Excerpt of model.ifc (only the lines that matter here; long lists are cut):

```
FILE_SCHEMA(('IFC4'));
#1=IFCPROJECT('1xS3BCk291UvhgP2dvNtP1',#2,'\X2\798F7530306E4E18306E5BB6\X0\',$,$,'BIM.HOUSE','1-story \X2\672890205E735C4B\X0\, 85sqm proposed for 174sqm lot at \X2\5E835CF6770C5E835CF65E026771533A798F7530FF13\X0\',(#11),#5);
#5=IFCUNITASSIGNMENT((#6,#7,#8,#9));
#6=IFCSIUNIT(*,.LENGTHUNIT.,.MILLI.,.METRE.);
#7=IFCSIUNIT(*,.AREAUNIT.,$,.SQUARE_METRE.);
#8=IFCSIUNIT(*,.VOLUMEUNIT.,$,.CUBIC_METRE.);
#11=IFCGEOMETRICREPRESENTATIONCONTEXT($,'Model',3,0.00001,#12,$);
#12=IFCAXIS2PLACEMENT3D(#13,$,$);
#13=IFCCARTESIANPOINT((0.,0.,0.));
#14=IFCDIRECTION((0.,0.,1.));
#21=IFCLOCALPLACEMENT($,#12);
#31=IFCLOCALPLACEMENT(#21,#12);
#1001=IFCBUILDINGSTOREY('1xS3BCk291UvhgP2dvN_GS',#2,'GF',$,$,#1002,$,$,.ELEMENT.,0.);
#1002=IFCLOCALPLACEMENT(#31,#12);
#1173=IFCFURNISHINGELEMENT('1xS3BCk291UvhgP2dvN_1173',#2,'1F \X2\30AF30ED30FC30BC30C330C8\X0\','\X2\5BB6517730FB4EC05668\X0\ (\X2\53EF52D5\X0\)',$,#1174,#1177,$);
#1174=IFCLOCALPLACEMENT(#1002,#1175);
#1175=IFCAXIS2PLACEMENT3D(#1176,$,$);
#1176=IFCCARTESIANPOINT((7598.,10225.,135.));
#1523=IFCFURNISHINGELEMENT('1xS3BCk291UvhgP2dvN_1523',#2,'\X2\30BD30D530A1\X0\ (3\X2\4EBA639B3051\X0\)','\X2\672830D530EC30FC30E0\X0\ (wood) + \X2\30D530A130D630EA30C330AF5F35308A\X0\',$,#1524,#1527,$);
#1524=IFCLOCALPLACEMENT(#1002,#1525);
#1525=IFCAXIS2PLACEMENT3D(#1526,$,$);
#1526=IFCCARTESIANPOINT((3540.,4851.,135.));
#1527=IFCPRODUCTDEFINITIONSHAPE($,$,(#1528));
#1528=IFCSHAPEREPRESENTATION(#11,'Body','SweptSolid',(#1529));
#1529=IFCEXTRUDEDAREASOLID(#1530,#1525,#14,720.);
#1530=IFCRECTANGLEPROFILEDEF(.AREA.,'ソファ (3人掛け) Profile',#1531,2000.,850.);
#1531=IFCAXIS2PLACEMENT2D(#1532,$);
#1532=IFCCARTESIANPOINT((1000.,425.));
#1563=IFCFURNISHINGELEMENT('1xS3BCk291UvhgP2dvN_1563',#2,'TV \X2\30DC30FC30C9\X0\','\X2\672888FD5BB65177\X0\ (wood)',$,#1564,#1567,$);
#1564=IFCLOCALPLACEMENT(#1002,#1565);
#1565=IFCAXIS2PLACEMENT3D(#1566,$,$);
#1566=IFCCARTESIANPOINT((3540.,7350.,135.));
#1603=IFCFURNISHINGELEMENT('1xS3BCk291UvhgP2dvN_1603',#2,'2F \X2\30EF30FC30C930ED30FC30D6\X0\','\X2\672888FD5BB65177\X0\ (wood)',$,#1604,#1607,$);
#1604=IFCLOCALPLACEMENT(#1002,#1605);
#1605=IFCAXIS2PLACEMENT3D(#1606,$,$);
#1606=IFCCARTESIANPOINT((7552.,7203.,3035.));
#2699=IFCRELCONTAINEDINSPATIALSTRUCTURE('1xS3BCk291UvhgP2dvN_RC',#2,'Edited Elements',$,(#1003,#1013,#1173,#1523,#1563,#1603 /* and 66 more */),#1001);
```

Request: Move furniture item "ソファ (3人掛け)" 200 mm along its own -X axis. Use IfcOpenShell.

```python
import ifcopenshell
import ifcopenshell.api.geometry
import ifcopenshell.util.placement
import ifcopenshell.util.unit

model = ifcopenshell.open("model.ifc")
unit_scale = ifcopenshell.util.unit.calculate_unit_scale(model)

item = model.by_guid("1xS3BCk291UvhgP2dvN_1523")
matrix = ifcopenshell.util.placement.get_local_placement(item.ObjectPlacement)
matrix[:3, 3] -= matrix[:3, 0] * 0.2 / unit_scale
ifcopenshell.api.geometry.edit_object_placement(model, product=item, matrix=matrix, is_si=False)

print(ifcopenshell.util.placement.get_local_placement(item.ObjectPlacement).round(3) + 0.0)

model.write("model_rev.ifc")
```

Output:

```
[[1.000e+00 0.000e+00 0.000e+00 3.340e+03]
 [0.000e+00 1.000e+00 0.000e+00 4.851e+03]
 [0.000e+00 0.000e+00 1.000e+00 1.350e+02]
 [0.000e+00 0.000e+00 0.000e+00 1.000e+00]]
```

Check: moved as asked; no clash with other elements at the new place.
